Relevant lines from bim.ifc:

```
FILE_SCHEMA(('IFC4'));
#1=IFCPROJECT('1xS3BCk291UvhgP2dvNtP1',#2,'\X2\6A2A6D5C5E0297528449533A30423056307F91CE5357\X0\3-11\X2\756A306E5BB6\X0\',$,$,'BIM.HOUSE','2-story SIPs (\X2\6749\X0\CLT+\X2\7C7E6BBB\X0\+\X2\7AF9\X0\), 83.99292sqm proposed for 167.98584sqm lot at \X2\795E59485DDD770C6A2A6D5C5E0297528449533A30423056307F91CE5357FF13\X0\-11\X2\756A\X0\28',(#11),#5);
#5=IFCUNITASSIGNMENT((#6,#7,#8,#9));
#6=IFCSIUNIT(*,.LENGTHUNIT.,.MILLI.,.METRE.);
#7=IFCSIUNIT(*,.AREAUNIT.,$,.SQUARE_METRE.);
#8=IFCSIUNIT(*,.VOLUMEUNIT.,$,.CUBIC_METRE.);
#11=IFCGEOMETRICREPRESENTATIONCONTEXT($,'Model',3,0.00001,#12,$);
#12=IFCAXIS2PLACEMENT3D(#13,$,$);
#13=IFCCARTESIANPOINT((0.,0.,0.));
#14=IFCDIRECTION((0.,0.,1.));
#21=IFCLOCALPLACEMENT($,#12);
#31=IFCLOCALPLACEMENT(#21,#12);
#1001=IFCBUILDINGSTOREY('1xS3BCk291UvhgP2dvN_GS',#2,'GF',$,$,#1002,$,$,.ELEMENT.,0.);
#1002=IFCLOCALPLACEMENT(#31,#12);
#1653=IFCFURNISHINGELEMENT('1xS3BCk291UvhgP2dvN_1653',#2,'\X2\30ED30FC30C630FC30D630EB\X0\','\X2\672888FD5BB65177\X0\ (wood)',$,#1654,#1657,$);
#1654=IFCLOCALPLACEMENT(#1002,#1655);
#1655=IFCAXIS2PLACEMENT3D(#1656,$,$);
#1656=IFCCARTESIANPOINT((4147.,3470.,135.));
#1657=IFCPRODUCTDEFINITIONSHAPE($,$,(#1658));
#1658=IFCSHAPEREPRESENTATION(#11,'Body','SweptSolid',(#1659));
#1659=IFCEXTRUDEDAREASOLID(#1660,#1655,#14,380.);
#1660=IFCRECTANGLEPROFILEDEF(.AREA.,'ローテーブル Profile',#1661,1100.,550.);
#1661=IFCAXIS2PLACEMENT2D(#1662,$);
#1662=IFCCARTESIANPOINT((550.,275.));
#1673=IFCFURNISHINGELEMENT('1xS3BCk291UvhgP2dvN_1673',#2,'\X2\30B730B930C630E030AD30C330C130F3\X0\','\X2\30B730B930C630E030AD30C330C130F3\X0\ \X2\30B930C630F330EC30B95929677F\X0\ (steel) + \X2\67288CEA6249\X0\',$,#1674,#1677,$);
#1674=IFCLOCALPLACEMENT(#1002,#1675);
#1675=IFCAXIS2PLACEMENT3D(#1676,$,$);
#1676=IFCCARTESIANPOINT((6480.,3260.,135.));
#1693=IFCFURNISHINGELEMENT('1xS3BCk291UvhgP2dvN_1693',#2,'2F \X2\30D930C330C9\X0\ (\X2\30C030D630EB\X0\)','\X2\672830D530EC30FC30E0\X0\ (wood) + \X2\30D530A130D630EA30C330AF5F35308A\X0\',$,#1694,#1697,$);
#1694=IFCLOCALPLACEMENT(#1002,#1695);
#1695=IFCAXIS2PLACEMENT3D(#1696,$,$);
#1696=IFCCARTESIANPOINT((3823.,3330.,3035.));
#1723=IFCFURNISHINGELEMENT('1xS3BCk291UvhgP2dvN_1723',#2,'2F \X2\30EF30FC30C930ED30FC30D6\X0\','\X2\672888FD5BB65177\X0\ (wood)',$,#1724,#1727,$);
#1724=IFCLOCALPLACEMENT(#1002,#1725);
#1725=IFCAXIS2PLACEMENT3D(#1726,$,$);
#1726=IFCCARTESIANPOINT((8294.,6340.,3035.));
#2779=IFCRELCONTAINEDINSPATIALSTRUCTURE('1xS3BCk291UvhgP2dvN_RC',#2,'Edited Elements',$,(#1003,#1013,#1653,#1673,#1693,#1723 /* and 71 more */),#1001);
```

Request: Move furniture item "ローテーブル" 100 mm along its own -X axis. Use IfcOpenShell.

```python
import ifcopenshell
import ifcopenshell.api.geometry
import ifcopenshell.util.placement

model = ifcopenshell.open("bim.ifc")

item = model.by_guid("1xS3BCk291UvhgP2dvN_1653")
matrix = ifcopenshell.util.placement.get_local_placement(item.ObjectPlacement)
matrix[:3, 3] -= matrix[:3, 0] * 100.0
ifcopenshell.api.geometry.edit_object_placement(model, product=item, matrix=matrix, is_si=False)

print(ifcopenshell.util.placement.get_local_placement(item.ObjectPlacement).round(3) + 0.0)

model.write("bim-out.ifc")
```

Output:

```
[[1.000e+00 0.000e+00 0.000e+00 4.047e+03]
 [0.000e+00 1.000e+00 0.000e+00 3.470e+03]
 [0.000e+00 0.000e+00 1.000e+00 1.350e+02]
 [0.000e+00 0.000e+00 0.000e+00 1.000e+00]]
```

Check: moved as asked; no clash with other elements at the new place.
